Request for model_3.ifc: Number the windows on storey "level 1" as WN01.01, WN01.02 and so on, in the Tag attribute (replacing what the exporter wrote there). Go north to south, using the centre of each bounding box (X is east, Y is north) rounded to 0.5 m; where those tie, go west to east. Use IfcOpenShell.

First a look at what the model holds.

```python
import ifcopenshell
import ifcopenshell.util.element
import ifcopenshell.util.placement

model = ifcopenshell.open("model_3.ifc")
print(model.schema)
storey = next(s for s in model.by_type("IfcBuildingStorey") if s.Name == "level 1")
windows = [e for e in ifcopenshell.util.element.get_decomposition(storey) if e.is_a("IfcWindow")]
for e in sorted(windows, key=lambda e: e.id()):
    origin = ifcopenshell.util.placement.get_local_placement(e.ObjectPlacement)[:3, 3]
    print(e.id(), e.Tag, e.Name, origin.round(2) + 0.0, sep=" | ")
```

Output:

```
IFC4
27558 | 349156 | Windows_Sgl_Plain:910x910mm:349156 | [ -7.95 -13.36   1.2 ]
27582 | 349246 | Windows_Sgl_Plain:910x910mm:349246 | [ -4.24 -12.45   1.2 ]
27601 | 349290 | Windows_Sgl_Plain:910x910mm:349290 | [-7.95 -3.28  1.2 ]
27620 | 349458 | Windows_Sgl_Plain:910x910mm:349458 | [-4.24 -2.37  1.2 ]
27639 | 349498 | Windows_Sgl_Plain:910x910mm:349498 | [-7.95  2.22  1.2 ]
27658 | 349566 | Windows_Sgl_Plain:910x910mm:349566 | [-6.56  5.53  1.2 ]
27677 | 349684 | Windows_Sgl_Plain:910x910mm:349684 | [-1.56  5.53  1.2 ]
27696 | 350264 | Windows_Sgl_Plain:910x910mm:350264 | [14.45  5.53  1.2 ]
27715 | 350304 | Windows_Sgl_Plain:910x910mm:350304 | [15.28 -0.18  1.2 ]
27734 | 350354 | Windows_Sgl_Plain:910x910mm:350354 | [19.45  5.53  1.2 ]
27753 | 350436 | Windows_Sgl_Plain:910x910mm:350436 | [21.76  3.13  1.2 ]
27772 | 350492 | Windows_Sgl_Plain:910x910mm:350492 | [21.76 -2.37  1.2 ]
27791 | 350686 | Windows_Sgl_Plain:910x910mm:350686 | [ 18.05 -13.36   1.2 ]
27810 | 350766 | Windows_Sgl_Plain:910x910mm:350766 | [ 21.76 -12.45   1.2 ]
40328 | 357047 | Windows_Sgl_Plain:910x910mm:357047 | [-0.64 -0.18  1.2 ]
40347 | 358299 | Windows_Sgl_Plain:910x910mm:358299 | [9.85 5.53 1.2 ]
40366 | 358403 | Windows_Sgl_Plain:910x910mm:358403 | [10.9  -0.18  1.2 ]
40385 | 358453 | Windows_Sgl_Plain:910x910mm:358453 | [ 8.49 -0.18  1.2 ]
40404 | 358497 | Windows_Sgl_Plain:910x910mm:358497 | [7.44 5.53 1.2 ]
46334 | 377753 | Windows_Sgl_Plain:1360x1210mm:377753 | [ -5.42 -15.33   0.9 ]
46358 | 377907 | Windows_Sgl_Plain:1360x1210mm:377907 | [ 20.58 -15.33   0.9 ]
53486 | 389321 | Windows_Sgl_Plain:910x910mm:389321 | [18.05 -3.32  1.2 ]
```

```python
import ifcopenshell
import ifcopenshell.geom
import ifcopenshell.util.element
import ifcopenshell.util.shape

model = ifcopenshell.open("model_3.ifc")
settings = ifcopenshell.geom.settings()
settings.set("use-world-coords", True)


def centre(element):
    shape = ifcopenshell.geom.create_shape(settings, element)
    return ifcopenshell.util.shape.get_bbox_centroid(shape.geometry)


storey = next(s for s in model.by_type("IfcBuildingStorey") if s.Name == "level 1")
windows = [e for e in ifcopenshell.util.element.get_decomposition(storey) if e.is_a("IfcWindow")]

# Insertion points can sit at a corner or the storey origin, so sort by the geometry (in metres).
centres = {e: centre(e) for e in windows}
windows.sort(key=lambda e: (-round(centres[e][1] / 0.5), centres[e][0]))

for i, e in enumerate(windows, start=1):
    number = f"WN01.{i:02d}"
    e.Tag = number
    print(e.id(), number)

model.write("model_3-out.ifc")
```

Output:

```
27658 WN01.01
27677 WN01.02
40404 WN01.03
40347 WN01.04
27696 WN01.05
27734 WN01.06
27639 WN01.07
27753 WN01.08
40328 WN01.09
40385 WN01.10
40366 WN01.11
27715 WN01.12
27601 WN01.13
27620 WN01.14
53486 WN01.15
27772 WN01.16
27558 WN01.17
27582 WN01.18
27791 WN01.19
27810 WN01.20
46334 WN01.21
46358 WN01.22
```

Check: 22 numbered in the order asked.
